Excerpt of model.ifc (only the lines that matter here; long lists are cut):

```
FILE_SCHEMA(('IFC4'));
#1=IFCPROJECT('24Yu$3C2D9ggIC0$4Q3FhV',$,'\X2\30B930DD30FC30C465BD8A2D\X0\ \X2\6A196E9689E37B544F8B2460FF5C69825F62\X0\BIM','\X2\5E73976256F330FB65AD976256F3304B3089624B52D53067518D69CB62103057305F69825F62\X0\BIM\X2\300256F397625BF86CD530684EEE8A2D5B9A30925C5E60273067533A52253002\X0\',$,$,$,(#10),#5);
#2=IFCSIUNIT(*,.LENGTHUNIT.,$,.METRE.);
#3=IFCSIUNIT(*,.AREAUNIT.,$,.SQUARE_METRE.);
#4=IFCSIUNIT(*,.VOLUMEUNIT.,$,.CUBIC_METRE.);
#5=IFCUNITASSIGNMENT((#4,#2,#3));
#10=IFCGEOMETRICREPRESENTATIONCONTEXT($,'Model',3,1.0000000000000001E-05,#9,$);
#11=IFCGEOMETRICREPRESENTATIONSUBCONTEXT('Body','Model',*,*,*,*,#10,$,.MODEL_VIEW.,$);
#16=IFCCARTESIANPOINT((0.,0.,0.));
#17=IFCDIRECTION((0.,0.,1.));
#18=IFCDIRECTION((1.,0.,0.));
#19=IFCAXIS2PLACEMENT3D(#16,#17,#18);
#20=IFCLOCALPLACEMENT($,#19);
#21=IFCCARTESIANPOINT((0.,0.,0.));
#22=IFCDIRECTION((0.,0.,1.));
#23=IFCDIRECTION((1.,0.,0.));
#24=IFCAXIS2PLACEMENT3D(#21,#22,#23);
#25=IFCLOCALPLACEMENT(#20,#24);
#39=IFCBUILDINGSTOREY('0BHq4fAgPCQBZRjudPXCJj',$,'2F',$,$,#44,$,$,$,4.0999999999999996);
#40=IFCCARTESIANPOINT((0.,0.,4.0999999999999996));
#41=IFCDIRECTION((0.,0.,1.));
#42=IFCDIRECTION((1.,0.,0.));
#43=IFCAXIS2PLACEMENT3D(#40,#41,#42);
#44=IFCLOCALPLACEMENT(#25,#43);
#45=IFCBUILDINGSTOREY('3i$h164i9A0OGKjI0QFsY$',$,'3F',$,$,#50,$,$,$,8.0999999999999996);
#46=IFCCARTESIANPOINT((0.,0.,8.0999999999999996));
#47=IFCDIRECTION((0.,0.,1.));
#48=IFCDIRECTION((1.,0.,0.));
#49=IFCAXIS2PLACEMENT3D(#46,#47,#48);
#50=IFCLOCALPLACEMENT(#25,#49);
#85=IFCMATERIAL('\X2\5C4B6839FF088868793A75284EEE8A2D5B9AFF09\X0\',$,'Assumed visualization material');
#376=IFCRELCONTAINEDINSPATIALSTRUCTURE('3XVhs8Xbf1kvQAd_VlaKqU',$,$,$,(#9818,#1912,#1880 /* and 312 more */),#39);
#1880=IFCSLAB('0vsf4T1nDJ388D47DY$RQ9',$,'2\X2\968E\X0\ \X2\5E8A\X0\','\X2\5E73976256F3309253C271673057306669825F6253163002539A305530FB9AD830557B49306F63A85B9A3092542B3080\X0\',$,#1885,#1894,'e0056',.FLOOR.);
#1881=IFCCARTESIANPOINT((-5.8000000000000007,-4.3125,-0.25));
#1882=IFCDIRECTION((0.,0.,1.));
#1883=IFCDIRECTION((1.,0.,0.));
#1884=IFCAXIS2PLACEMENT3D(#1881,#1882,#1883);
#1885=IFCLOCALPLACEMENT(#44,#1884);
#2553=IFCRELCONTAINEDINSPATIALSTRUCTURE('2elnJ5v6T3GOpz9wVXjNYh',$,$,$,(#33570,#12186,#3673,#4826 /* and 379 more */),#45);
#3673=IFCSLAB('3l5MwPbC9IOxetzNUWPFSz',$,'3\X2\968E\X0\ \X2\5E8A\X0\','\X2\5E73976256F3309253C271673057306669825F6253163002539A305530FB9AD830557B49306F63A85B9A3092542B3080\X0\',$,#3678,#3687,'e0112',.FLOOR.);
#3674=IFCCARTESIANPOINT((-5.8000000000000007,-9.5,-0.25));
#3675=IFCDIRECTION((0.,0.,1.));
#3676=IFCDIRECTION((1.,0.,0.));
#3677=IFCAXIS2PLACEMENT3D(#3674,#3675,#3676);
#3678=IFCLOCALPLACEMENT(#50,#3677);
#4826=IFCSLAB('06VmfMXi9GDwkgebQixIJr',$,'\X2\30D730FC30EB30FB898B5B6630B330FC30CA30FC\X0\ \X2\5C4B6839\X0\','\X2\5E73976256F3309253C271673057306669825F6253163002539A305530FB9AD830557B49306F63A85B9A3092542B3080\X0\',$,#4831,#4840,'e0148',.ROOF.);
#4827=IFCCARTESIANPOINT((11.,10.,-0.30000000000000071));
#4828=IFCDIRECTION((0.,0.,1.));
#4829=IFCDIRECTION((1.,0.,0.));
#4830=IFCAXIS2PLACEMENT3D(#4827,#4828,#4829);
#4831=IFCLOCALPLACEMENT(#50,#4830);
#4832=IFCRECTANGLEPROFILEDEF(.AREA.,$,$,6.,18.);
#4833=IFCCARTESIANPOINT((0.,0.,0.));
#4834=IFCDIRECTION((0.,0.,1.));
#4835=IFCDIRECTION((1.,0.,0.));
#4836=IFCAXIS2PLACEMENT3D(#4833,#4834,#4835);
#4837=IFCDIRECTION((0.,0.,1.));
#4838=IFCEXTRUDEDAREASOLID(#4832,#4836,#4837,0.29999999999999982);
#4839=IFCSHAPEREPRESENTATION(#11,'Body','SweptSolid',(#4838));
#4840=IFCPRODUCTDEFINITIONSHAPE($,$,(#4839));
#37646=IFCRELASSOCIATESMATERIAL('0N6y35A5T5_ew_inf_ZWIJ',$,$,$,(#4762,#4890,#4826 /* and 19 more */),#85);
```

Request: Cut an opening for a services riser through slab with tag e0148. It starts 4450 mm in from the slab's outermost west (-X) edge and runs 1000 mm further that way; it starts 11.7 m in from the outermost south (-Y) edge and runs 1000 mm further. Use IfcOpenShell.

```python
import numpy as np
import ifcopenshell
import ifcopenshell.api.feature
import ifcopenshell.api.geometry
import ifcopenshell.api.root
import ifcopenshell.geom
import ifcopenshell.util.placement
import ifcopenshell.util.representation
import ifcopenshell.util.shape
import ifcopenshell.util.unit

model = ifcopenshell.open("model.ifc")
unit_scale = ifcopenshell.util.unit.calculate_unit_scale(model)
settings = ifcopenshell.geom.settings()


def volume(element):
    """Net volume in cubic metres, openings subtracted."""
    shape = ifcopenshell.geom.create_shape(settings, element)
    return ifcopenshell.util.shape.get_volume(shape.geometry)


slab = model.by_guid("06VmfMXi9GDwkgebQixIJr")
before = volume(slab)

# Extent in the slab's own axes, in metres. The edges named are its -X and -Y sides.
slab_shape = ifcopenshell.geom.create_shape(settings, slab)
vertices = ifcopenshell.util.shape.get_vertices(slab_shape.geometry)
x_min, y_min, bottom = vertices.min(axis=0)
top = vertices[:, 2].max()

opening = ifcopenshell.api.root.create_entity(model, ifc_class="IfcOpeningElement", name="Services riser opening", predefined_type="OPENING")
context = ifcopenshell.util.representation.get_context(model, "Model", "Body", "MODEL_VIEW")
width, depth = 1, 1
outline = [(0.0, 0.0), (width, 0.0), (width, depth), (0.0, depth), (0.0, 0.0)]
# Overshoot both faces by 50 mm so the cut is clean.
shape = ifcopenshell.api.geometry.add_slab_representation(
    model, context=context, depth=top - bottom + 0.1, polyline=outline
)
ifcopenshell.api.geometry.assign_representation(model, product=opening, representation=shape)

matrix = ifcopenshell.util.placement.get_local_placement(slab.ObjectPlacement)
matrix[:, 3] = matrix @ np.append(np.array([x_min + 4.45, y_min + 11.7, bottom - 0.05]) / unit_scale, 1.0)
ifcopenshell.api.geometry.edit_object_placement(model, product=opening, matrix=matrix, is_si=False)
ifcopenshell.api.feature.add_feature(model, feature=opening, element=slab)

after = volume(slab)

print(f"slab volume {before:.3f} -> {after:.3f} m3")

model.write("model_rev.ifc")
```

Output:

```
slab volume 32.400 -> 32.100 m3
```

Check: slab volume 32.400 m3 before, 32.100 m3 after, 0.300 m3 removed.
